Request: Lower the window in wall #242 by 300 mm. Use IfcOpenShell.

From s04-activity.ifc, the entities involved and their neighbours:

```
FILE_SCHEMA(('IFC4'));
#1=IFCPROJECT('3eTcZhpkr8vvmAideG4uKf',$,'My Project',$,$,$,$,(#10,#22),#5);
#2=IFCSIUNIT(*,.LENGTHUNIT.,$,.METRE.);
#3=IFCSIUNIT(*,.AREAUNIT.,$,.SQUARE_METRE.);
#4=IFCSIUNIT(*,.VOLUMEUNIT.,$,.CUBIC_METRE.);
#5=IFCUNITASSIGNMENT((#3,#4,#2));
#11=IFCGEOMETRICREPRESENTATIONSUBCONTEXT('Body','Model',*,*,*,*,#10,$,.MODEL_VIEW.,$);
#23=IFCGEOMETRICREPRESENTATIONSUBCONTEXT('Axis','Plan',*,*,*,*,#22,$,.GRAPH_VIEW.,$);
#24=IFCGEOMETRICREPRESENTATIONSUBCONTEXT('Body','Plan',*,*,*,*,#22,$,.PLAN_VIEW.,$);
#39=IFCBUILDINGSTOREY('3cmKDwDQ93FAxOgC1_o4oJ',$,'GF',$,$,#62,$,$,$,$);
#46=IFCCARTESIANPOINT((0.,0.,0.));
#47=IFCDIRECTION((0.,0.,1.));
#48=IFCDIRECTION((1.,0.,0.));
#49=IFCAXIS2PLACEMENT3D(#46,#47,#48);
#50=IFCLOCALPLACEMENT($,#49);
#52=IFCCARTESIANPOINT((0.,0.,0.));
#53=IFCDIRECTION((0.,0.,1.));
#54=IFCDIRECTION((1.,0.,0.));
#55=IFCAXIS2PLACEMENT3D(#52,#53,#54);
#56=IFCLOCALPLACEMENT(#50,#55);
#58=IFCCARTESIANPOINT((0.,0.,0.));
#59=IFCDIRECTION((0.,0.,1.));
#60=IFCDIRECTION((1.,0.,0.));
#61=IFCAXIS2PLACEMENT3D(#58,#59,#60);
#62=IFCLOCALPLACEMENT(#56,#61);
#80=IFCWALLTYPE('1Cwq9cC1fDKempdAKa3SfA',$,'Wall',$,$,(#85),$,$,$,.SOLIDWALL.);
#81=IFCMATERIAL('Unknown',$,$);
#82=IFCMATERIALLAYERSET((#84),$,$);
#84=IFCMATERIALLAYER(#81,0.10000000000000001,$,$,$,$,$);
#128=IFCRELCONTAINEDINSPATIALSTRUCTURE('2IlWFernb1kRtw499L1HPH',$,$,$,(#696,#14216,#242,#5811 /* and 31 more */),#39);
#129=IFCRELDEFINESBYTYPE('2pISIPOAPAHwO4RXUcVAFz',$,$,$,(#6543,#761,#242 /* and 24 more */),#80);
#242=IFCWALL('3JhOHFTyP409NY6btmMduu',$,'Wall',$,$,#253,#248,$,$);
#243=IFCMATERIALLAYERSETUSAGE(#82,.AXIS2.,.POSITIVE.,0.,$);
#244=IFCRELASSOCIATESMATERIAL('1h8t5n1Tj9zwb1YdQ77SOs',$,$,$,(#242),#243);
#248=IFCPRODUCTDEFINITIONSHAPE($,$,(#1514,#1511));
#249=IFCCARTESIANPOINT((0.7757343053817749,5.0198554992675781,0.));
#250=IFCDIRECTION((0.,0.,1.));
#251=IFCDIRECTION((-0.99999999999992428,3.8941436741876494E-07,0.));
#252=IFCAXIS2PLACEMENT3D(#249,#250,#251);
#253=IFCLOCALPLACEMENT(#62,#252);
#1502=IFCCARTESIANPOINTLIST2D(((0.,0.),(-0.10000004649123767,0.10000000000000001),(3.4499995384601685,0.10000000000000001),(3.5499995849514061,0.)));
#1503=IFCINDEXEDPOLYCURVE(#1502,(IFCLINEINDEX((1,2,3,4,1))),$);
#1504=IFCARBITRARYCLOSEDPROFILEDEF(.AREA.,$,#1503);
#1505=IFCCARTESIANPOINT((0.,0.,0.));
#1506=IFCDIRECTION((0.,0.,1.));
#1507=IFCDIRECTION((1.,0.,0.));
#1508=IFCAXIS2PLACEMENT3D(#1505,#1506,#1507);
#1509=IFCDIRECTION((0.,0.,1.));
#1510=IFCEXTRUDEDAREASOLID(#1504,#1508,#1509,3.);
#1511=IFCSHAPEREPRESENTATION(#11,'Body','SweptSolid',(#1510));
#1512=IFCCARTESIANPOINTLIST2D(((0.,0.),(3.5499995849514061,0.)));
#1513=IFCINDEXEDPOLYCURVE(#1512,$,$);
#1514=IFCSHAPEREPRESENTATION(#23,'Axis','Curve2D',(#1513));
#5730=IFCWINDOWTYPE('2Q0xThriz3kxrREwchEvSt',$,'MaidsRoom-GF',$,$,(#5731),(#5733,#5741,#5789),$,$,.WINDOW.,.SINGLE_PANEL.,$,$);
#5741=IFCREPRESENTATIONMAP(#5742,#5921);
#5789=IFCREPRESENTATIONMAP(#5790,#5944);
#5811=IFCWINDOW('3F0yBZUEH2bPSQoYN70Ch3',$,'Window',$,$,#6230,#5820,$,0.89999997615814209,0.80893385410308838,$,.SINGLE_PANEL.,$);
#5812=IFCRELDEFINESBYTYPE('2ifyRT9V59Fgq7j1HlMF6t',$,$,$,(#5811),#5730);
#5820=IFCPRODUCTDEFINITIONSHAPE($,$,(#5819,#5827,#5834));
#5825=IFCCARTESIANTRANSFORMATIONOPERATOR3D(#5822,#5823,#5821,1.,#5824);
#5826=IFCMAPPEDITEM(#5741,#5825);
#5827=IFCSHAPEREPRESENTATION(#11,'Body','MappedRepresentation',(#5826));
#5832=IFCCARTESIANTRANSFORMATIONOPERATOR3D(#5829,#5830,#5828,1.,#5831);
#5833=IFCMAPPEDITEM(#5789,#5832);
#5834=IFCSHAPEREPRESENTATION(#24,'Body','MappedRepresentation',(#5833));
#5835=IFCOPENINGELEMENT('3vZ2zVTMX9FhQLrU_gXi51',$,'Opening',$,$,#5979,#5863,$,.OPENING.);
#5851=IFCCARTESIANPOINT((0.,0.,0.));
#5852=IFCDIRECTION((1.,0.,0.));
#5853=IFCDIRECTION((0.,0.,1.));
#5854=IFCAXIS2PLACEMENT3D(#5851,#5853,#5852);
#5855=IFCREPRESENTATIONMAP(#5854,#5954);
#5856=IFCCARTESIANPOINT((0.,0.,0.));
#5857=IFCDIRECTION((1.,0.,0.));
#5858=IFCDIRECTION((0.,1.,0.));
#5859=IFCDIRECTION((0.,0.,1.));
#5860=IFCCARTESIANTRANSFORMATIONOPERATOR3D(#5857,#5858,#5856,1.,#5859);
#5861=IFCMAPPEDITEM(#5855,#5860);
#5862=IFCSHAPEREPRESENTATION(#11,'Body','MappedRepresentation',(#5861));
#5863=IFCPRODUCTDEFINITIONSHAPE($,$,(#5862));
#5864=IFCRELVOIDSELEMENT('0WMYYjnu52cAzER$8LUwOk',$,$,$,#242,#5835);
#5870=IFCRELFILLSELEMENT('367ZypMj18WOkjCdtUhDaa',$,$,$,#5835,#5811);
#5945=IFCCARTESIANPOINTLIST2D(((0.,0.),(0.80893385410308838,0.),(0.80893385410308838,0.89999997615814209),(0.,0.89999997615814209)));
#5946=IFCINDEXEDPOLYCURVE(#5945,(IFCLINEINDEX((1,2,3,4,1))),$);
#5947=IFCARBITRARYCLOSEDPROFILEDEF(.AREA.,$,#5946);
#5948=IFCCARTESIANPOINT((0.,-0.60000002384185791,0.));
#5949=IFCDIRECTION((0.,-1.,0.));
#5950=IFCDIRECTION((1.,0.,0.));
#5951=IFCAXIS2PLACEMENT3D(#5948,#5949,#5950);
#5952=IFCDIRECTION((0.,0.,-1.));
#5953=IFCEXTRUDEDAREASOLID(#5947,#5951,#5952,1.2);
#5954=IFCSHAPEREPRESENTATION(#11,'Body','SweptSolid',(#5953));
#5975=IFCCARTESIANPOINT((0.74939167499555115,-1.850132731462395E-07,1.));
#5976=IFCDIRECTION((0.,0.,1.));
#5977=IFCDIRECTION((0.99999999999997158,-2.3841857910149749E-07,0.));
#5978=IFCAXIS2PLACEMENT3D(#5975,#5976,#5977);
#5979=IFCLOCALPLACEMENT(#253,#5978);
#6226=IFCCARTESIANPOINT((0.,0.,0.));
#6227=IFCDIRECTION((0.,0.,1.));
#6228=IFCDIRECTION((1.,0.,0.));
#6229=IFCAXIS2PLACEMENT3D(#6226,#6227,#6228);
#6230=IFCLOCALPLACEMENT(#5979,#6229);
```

```python
import numpy as np
import ifcopenshell
import ifcopenshell.api.geometry
import ifcopenshell.util.placement
import ifcopenshell.util.unit

model = ifcopenshell.open("s04-activity.ifc")
unit_scale = ifcopenshell.util.unit.calculate_unit_scale(model)

window = model.by_guid("3F0yBZUEH2bPSQoYN70Ch3")
opening = window.FillsVoids[0].RelatingOpeningElement
dz = -0.3

shift = np.array([0.0, 0.0, dz])
# The window is placed relative to its opening, so it follows when the opening moves.
matrix = ifcopenshell.util.placement.get_local_placement(opening.ObjectPlacement)
matrix[:3, 3] += shift
ifcopenshell.api.geometry.edit_object_placement(
    model, product=opening, matrix=matrix, is_si=False, should_transform_children=True
)

print(f"moved by {dz * unit_scale:+.3f} m")

model.write("s04-activity_updated.ifc")
```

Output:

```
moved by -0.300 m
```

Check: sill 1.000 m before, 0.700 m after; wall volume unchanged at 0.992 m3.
